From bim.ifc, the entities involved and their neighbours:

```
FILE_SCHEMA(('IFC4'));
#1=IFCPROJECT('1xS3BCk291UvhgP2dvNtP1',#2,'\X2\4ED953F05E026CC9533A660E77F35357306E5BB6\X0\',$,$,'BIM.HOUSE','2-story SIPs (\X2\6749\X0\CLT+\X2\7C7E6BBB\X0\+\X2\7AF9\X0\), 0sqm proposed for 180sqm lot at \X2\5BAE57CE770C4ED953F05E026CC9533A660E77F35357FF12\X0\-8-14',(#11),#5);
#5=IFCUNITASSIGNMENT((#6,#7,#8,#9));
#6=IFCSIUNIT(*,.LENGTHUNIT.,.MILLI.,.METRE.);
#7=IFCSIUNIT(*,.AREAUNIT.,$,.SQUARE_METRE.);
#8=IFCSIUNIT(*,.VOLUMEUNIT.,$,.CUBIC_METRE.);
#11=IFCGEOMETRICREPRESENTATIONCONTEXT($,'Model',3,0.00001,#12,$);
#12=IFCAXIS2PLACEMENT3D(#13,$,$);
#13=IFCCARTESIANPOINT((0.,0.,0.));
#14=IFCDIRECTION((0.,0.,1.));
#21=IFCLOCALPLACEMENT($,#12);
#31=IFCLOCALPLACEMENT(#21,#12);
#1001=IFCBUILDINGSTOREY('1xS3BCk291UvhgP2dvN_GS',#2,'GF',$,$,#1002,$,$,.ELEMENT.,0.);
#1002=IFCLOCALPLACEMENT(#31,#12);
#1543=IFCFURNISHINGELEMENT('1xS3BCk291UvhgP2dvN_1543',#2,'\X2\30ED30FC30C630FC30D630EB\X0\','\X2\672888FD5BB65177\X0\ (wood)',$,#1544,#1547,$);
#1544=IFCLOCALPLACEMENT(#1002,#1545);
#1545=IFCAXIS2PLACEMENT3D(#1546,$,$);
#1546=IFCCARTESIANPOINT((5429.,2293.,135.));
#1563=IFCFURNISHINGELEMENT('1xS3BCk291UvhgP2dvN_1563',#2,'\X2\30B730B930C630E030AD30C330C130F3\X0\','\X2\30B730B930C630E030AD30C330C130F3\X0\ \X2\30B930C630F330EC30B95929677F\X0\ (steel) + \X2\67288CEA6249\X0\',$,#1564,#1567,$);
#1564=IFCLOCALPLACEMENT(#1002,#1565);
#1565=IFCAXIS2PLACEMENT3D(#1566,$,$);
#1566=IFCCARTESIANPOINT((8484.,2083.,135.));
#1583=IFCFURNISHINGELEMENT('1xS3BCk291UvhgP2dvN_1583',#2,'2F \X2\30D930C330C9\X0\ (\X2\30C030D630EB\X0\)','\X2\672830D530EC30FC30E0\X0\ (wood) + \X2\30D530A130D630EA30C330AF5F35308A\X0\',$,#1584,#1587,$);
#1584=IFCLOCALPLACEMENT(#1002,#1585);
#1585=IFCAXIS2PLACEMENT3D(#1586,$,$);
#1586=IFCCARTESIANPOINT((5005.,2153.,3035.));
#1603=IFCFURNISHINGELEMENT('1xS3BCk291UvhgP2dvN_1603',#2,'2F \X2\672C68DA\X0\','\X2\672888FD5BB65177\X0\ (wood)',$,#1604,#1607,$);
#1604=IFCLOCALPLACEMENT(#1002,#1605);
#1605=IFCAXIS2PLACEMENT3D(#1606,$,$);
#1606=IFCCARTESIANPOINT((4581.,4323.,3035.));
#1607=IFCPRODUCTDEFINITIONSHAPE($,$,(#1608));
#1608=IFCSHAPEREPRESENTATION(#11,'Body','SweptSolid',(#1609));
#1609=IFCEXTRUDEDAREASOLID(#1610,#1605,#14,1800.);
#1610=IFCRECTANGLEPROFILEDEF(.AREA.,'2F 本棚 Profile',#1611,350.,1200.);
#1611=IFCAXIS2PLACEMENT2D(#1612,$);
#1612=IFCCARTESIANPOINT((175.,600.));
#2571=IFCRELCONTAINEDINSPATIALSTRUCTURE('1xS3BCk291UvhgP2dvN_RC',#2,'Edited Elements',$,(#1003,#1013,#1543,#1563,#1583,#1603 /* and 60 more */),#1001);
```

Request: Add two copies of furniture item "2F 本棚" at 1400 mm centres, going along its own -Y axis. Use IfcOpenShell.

```python
import ifcopenshell
import ifcopenshell.api.geometry
import ifcopenshell.api.root
import ifcopenshell.util.element
import ifcopenshell.util.placement
import ifcopenshell.util.unit

model = ifcopenshell.open("bim.ifc")
unit_scale = ifcopenshell.util.unit.calculate_unit_scale(model)


def reuse_history(source, copy):
    """copy_class also copies each property set's owner history, people and application; keep the originals."""
    for rel in copy.IsDefinedBy:
        if rel.is_a("IfcRelDefinesByProperties") and (history := rel.RelatingPropertyDefinition.OwnerHistory):
            rel.RelatingPropertyDefinition.OwnerHistory = source.OwnerHistory
            ifcopenshell.util.element.remove_deep2(model, history)


source = model.by_id(1603)
base = ifcopenshell.util.placement.get_local_placement(source.ObjectPlacement)
step = -base[:3, 1] * 1.4 / unit_scale

for i in range(1, 3):
    copy = ifcopenshell.api.root.copy_class(model, product=source)
    copy.Representation = ifcopenshell.util.element.copy_deep(
        model, source.Representation, exclude=["IfcGeometricRepresentationContext", "IfcRepresentationMap"]
    )
    reuse_history(source, copy)
    matrix = base.copy()
    matrix[:3, 3] += i * step
    print("added at", matrix[:3, 3].round(3) + 0.0)
    ifcopenshell.api.geometry.edit_object_placement(model, product=copy, matrix=matrix, is_si=False)

model.write("bim_updated.ifc")
```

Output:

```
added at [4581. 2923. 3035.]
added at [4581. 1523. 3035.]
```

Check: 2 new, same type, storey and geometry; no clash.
